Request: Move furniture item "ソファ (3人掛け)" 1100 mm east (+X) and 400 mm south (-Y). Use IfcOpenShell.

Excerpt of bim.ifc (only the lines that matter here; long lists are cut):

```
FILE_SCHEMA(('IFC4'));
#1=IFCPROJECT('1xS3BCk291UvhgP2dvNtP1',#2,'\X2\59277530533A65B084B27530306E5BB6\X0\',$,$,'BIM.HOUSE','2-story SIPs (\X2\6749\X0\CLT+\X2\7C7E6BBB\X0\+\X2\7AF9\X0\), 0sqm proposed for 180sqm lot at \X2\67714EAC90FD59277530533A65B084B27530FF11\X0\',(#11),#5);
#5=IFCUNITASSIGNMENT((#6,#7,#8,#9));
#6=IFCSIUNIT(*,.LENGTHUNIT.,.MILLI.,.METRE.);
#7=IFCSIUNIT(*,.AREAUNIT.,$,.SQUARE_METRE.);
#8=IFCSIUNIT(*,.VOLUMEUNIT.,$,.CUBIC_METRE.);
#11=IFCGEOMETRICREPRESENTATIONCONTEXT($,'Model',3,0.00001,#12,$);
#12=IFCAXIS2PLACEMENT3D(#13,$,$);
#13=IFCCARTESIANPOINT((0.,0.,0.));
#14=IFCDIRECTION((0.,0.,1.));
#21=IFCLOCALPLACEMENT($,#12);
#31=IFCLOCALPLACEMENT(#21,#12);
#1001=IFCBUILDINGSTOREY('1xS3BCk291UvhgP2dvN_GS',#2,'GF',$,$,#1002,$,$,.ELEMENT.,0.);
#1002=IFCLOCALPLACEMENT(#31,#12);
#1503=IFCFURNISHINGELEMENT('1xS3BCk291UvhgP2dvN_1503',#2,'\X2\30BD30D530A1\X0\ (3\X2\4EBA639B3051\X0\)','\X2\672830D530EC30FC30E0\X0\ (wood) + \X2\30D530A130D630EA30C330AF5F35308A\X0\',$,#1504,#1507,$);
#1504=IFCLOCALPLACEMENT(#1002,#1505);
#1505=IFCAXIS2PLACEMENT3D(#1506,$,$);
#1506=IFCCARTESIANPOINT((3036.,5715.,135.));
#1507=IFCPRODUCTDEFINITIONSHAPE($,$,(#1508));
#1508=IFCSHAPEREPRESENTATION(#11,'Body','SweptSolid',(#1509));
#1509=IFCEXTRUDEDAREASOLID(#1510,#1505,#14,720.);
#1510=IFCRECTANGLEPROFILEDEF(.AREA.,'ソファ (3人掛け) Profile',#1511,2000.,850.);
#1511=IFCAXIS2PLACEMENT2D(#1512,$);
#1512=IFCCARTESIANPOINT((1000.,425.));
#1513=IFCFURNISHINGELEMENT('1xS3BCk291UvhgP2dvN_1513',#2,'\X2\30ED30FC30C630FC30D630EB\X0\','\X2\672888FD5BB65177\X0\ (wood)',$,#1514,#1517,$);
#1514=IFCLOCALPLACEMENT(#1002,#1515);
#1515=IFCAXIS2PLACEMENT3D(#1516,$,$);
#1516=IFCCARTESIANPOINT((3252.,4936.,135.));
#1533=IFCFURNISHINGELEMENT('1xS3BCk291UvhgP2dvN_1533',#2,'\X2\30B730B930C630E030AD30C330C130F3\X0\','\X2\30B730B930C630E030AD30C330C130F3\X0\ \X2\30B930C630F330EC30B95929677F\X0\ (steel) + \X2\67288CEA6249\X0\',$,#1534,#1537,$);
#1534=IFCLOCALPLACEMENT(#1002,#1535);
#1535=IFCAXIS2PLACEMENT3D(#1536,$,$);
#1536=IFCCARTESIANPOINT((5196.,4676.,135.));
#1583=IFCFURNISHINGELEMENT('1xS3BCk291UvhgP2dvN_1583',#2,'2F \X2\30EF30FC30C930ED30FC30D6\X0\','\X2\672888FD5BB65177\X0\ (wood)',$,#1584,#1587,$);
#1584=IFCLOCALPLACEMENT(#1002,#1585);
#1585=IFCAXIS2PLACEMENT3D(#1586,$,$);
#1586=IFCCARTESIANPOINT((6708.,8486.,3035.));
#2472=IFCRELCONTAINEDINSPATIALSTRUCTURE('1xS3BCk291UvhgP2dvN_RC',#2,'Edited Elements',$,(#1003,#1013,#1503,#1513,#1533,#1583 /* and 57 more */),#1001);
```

```python
import ifcopenshell
import ifcopenshell.api.geometry
import ifcopenshell.util.placement
import ifcopenshell.util.unit

model = ifcopenshell.open("bim.ifc")
unit_scale = ifcopenshell.util.unit.calculate_unit_scale(model)

item = model.by_id(1503)
matrix = ifcopenshell.util.placement.get_local_placement(item.ObjectPlacement)
matrix[0, 3] += 1.1 / unit_scale
matrix[1, 3] -= 0.4 / unit_scale
ifcopenshell.api.geometry.edit_object_placement(model, product=item, matrix=matrix, is_si=False)

print(ifcopenshell.util.placement.get_local_placement(item.ObjectPlacement).round(3) + 0.0)

model.write("bim-out.ifc")
```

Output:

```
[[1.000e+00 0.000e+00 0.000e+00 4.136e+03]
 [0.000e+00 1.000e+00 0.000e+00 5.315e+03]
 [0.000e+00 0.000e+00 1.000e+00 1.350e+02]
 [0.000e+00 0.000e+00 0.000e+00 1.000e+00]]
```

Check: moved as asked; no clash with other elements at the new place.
